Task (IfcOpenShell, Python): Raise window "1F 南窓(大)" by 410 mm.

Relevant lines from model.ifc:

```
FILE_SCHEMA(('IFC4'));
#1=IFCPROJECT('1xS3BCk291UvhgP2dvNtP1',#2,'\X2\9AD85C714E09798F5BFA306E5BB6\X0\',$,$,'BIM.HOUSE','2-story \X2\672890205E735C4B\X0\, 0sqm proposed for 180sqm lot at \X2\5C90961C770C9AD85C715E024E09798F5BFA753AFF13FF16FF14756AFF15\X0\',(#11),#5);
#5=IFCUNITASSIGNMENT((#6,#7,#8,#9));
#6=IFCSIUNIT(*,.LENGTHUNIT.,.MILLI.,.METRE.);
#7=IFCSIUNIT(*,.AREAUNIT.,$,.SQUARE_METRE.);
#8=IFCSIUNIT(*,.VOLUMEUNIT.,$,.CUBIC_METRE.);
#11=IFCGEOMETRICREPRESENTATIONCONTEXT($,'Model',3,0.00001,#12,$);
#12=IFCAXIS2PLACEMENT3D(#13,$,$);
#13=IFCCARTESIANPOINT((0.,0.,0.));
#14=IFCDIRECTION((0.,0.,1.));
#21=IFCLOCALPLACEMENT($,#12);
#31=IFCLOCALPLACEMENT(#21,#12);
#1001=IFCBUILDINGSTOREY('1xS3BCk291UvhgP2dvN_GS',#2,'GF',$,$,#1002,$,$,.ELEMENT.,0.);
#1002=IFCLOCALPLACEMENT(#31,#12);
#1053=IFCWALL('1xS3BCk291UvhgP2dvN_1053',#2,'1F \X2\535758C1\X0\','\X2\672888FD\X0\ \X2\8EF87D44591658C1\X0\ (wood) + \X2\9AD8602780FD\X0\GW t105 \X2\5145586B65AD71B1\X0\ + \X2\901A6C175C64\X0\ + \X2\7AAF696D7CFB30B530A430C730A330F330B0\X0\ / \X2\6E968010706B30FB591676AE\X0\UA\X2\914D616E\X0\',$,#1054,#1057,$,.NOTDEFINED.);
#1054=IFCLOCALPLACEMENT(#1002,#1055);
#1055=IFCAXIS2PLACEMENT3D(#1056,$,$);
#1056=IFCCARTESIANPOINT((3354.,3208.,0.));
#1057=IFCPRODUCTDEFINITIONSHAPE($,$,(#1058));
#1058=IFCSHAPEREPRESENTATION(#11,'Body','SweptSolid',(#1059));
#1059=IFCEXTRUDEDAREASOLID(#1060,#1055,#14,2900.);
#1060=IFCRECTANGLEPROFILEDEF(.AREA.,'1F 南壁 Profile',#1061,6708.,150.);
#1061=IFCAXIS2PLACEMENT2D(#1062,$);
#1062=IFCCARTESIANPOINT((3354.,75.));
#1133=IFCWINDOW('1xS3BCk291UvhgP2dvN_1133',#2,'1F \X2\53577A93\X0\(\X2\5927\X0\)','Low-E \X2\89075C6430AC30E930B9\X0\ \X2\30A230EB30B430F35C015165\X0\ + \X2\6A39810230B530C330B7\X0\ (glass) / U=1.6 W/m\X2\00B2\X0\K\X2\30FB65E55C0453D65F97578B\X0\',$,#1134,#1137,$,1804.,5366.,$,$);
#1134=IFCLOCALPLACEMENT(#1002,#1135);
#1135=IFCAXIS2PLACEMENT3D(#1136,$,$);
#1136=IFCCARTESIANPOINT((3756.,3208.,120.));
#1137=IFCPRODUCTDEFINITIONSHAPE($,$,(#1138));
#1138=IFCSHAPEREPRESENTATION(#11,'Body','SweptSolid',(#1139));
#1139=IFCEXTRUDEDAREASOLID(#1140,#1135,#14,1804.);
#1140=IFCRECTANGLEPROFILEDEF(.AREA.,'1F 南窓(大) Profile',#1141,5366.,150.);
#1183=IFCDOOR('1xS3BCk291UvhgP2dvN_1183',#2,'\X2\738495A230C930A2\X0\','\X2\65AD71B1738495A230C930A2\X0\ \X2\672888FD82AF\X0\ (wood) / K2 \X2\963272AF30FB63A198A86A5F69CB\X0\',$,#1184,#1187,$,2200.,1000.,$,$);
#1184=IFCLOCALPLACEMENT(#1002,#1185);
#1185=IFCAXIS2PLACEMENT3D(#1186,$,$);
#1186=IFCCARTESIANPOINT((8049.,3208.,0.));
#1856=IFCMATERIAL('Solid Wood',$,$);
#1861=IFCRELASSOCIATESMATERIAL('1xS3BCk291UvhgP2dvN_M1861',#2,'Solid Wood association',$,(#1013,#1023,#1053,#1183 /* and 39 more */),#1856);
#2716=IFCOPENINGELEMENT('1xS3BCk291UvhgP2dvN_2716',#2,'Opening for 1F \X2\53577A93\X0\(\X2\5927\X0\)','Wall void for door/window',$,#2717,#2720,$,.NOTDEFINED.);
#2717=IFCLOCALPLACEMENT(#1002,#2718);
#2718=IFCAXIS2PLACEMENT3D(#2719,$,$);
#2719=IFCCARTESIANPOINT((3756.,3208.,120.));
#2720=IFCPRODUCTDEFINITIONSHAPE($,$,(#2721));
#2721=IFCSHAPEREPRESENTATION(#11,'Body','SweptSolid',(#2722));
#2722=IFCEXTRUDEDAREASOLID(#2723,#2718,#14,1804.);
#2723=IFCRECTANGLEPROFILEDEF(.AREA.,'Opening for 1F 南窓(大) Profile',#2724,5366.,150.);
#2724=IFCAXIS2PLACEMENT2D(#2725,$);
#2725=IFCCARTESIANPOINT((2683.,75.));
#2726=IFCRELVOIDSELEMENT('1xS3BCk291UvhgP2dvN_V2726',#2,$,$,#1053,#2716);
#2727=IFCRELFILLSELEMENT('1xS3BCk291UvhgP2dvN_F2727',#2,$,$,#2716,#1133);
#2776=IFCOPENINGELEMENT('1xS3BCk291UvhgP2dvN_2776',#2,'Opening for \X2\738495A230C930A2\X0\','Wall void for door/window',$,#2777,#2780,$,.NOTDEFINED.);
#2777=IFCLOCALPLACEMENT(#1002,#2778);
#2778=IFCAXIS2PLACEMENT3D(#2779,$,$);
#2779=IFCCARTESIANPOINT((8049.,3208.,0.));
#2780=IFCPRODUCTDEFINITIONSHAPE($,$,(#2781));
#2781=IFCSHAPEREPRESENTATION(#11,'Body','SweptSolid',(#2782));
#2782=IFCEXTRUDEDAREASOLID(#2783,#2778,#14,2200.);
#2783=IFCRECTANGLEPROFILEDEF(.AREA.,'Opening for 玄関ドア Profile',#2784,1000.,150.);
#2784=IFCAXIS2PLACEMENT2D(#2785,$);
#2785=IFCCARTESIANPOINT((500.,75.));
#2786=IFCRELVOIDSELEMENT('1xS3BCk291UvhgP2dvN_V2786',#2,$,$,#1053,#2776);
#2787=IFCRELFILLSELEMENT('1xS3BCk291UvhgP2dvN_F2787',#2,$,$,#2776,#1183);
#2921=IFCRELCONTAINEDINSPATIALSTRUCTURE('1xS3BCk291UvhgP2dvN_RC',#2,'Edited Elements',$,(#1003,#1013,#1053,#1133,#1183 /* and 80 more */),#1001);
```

```python
import numpy as np
import ifcopenshell
import ifcopenshell.api.geometry
import ifcopenshell.util.placement
import ifcopenshell.util.unit

model = ifcopenshell.open("model.ifc")
unit_scale = ifcopenshell.util.unit.calculate_unit_scale(model)

window = model.by_guid("1xS3BCk291UvhgP2dvN_1133")
opening = window.FillsVoids[0].RelatingOpeningElement
dz = 0.41 / unit_scale

shift = np.array([0.0, 0.0, dz])
# The window is not placed relative to its opening, so move both.
for product in (opening, window):
    matrix = ifcopenshell.util.placement.get_local_placement(product.ObjectPlacement)
    matrix[:3, 3] += shift
    ifcopenshell.api.geometry.edit_object_placement(model, product=product, matrix=matrix, is_si=False)

print(f"moved by {dz * unit_scale:+.3f} m")

model.write("model_edited.ifc")
```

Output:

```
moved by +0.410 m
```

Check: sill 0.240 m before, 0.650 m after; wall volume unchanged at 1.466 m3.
